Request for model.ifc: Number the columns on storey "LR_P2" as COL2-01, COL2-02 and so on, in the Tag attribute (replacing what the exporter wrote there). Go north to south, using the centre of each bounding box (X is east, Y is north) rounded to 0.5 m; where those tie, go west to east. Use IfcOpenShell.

First a look at what the model holds.

```python
import ifcopenshell
import ifcopenshell.util.element
import ifcopenshell.util.placement

model = ifcopenshell.open("model.ifc")
print(model.schema)
storey = next(s for s in model.by_type("IfcBuildingStorey") if s.Name == "LR_P2")
columns = [e for e in ifcopenshell.util.element.get_decomposition(storey) if e.is_a("IfcColumn")]
for e in sorted(columns, key=lambda e: e.id()):
    origin = ifcopenshell.util.placement.get_local_placement(e.ObjectPlacement)[:3, 3]
    print(e.id(), e.Tag, e.Name, origin.round(2) + 0.0, sep=" | ")
```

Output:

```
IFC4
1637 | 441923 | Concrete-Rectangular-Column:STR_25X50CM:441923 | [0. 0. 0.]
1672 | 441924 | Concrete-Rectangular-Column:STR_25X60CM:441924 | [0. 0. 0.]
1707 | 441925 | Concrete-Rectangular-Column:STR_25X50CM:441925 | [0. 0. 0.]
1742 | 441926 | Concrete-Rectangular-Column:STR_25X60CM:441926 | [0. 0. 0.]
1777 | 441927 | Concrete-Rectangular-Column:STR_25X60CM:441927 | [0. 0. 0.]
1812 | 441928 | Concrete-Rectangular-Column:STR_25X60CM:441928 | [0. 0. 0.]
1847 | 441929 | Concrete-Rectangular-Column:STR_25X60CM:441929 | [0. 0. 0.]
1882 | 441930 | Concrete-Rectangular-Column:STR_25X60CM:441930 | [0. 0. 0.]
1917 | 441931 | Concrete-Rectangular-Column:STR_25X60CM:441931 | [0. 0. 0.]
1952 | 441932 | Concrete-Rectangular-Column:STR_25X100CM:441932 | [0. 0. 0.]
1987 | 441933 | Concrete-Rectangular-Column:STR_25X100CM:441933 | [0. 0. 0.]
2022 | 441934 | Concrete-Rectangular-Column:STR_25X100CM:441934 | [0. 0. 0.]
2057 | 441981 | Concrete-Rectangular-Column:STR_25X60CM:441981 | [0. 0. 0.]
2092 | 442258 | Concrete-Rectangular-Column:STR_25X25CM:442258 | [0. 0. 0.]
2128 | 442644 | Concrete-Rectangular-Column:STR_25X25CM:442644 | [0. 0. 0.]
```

```python
import ifcopenshell
import ifcopenshell.geom
import ifcopenshell.util.element
import ifcopenshell.util.shape

model = ifcopenshell.open("model.ifc")
settings = ifcopenshell.geom.settings()
settings.set("use-world-coords", True)


def centre(element):
    shape = ifcopenshell.geom.create_shape(settings, element)
    return ifcopenshell.util.shape.get_bbox_centroid(shape.geometry)


storey = next(s for s in model.by_type("IfcBuildingStorey") if s.Name == "LR_P2")
columns = [e for e in ifcopenshell.util.element.get_decomposition(storey) if e.is_a("IfcColumn")]

# Insertion points can sit at a corner or the storey origin, so sort by the geometry (in metres).
centres = {e: centre(e) for e in columns}
columns.sort(key=lambda e: (-round(centres[e][1] / 0.5), centres[e][0]))

for i, e in enumerate(columns, start=1):
    number = f"COL2-{i:02d}"
    e.Tag = number
    print(e.id(), number)

model.write("model_rev.ifc")
```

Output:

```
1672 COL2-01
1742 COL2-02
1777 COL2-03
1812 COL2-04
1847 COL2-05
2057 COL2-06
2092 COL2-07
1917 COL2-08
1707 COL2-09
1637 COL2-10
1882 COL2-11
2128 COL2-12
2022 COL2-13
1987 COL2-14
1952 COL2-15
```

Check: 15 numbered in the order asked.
